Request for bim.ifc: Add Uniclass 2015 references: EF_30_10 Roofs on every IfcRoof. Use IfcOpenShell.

First a look at what the model holds.

```python
import ifcopenshell

model = ifcopenshell.open("bim.ifc")
print(model.schema)
print("classifications:", [c.Name for c in model.by_type("IfcClassification")])
for ifc_class in ("IfcDoor", "IfcRoof", "IfcStair", "IfcWall", "IfcWindow"):
    print(ifc_class, len(model.by_type(ifc_class)))
```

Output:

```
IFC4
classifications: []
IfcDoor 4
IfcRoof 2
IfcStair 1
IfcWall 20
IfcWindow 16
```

```python
import ifcopenshell
import ifcopenshell.api.classification

model = ifcopenshell.open("bim.ifc")

system = ifcopenshell.api.classification.add_classification(model, classification="Uniclass 2015")

codes = {
    "IfcRoof": ("EF_30_10", "Roofs"),
}
for ifc_class, (code, name) in codes.items():
    products = model.by_type(ifc_class)
    ifcopenshell.api.classification.add_reference(
        model, products=products, classification=system, identification=code, name=name
    )
    print(code, len(products))

model.write("bim-out.ifc")
```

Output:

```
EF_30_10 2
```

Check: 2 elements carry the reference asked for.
